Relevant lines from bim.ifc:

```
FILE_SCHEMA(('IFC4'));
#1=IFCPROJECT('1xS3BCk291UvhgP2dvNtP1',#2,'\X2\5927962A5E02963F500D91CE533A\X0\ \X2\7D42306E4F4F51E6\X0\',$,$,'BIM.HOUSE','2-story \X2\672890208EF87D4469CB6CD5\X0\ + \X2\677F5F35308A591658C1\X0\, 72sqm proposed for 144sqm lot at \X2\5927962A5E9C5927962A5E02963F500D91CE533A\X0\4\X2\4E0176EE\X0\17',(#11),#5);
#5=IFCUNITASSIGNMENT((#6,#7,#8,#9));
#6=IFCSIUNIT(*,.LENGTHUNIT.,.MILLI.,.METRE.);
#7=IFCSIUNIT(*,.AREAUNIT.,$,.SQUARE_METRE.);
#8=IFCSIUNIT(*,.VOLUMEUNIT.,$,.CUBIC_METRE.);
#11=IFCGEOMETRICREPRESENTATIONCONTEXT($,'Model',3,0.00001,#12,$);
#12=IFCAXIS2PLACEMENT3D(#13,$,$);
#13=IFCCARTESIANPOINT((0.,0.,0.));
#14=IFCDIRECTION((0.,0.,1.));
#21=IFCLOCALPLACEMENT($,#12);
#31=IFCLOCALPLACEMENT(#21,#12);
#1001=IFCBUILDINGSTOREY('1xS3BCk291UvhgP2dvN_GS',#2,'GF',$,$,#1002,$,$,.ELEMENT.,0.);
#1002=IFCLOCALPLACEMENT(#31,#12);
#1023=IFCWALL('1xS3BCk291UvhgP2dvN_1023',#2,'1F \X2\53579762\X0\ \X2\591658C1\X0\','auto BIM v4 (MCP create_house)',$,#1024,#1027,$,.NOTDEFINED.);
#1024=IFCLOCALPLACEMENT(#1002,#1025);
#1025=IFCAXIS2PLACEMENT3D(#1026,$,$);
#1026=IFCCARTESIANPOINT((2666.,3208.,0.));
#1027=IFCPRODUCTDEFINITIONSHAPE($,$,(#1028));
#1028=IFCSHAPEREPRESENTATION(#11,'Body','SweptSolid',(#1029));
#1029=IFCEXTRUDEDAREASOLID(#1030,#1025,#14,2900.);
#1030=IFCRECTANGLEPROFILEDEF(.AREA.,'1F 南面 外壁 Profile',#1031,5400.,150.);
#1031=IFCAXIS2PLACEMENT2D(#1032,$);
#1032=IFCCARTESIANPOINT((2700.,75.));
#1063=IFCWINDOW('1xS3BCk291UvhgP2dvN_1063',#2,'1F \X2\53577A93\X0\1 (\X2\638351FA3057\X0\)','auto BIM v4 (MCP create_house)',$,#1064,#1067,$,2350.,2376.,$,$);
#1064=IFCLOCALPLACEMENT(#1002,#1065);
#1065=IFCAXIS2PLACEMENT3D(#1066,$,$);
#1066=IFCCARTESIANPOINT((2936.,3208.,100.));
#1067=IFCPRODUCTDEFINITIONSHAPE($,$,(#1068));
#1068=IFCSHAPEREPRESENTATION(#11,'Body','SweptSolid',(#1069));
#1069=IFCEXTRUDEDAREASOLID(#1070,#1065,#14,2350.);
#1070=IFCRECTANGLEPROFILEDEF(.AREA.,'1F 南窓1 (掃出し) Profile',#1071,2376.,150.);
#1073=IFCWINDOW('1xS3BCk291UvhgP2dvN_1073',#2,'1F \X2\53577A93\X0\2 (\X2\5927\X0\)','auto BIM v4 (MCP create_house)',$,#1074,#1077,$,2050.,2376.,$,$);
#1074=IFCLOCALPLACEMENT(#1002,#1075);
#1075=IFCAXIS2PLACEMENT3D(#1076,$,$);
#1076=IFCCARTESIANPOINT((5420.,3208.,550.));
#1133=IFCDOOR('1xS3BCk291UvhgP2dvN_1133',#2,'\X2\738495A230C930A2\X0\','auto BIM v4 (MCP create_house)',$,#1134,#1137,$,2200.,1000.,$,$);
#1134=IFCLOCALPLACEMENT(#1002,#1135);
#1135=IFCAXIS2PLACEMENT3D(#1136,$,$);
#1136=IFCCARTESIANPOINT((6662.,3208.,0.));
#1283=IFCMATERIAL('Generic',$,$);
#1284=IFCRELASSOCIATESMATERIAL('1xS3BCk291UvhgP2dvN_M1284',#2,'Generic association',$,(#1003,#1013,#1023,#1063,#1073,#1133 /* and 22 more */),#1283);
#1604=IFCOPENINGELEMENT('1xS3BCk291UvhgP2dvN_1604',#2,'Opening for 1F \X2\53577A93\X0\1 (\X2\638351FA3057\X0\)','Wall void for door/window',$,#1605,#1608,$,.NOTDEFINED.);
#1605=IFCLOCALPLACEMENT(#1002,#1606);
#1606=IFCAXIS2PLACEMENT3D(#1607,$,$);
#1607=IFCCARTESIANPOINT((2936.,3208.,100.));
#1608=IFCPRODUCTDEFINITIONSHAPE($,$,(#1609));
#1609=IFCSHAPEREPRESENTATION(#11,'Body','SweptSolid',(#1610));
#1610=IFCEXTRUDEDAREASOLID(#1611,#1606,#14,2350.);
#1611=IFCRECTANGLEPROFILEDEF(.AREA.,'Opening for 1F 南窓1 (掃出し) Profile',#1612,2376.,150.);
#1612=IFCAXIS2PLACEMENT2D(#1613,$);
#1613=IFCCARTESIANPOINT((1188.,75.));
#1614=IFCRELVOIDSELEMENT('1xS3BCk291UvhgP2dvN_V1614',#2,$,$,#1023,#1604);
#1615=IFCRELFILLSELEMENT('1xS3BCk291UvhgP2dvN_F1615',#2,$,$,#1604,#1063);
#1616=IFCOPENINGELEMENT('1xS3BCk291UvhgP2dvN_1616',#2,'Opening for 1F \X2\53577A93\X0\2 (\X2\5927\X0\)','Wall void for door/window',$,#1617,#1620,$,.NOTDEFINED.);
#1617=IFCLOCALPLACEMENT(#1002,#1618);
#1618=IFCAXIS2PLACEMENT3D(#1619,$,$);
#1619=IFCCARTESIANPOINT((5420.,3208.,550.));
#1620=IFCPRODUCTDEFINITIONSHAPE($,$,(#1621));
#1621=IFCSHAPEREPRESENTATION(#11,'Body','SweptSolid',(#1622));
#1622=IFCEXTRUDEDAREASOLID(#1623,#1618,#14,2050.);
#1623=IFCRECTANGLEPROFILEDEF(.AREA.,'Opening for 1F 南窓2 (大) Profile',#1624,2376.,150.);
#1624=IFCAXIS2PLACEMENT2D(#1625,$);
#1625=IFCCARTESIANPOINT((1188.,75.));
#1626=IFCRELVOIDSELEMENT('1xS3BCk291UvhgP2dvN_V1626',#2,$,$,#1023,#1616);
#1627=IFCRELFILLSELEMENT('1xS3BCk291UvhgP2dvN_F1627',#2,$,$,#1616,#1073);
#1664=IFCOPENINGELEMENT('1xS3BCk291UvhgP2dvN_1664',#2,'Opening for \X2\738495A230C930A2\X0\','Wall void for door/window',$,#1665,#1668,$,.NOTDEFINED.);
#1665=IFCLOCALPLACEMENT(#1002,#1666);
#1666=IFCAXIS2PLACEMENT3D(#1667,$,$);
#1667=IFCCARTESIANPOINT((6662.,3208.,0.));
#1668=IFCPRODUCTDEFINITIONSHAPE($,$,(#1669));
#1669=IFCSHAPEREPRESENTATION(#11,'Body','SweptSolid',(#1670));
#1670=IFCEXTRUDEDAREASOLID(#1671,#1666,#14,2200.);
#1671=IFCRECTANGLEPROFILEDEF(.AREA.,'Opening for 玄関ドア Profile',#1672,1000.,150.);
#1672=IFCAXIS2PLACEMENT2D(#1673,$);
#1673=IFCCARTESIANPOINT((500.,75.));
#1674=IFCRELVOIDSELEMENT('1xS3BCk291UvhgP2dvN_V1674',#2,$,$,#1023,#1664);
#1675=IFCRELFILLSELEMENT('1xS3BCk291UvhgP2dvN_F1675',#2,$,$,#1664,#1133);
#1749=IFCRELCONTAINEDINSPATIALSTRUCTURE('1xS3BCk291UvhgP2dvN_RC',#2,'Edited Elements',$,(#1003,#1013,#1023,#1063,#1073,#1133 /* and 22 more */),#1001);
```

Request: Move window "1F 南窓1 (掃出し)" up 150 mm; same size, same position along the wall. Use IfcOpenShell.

```python
import numpy as np
import ifcopenshell
import ifcopenshell.api.geometry
import ifcopenshell.util.placement
import ifcopenshell.util.unit

model = ifcopenshell.open("bim.ifc")
unit_scale = ifcopenshell.util.unit.calculate_unit_scale(model)

window = model.by_id(1063)
opening = window.FillsVoids[0].RelatingOpeningElement
dz = 0.15 / unit_scale

shift = np.array([0.0, 0.0, dz])
# The window is not placed relative to its opening, so move both.
for product in (opening, window):
    matrix = ifcopenshell.util.placement.get_local_placement(product.ObjectPlacement)
    matrix[:3, 3] += shift
    ifcopenshell.api.geometry.edit_object_placement(model, product=product, matrix=matrix, is_si=False)

print(f"moved by {dz * unit_scale:+.3f} m")

model.write("bim_updated.ifc")
```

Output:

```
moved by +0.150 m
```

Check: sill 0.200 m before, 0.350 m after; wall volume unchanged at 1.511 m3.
